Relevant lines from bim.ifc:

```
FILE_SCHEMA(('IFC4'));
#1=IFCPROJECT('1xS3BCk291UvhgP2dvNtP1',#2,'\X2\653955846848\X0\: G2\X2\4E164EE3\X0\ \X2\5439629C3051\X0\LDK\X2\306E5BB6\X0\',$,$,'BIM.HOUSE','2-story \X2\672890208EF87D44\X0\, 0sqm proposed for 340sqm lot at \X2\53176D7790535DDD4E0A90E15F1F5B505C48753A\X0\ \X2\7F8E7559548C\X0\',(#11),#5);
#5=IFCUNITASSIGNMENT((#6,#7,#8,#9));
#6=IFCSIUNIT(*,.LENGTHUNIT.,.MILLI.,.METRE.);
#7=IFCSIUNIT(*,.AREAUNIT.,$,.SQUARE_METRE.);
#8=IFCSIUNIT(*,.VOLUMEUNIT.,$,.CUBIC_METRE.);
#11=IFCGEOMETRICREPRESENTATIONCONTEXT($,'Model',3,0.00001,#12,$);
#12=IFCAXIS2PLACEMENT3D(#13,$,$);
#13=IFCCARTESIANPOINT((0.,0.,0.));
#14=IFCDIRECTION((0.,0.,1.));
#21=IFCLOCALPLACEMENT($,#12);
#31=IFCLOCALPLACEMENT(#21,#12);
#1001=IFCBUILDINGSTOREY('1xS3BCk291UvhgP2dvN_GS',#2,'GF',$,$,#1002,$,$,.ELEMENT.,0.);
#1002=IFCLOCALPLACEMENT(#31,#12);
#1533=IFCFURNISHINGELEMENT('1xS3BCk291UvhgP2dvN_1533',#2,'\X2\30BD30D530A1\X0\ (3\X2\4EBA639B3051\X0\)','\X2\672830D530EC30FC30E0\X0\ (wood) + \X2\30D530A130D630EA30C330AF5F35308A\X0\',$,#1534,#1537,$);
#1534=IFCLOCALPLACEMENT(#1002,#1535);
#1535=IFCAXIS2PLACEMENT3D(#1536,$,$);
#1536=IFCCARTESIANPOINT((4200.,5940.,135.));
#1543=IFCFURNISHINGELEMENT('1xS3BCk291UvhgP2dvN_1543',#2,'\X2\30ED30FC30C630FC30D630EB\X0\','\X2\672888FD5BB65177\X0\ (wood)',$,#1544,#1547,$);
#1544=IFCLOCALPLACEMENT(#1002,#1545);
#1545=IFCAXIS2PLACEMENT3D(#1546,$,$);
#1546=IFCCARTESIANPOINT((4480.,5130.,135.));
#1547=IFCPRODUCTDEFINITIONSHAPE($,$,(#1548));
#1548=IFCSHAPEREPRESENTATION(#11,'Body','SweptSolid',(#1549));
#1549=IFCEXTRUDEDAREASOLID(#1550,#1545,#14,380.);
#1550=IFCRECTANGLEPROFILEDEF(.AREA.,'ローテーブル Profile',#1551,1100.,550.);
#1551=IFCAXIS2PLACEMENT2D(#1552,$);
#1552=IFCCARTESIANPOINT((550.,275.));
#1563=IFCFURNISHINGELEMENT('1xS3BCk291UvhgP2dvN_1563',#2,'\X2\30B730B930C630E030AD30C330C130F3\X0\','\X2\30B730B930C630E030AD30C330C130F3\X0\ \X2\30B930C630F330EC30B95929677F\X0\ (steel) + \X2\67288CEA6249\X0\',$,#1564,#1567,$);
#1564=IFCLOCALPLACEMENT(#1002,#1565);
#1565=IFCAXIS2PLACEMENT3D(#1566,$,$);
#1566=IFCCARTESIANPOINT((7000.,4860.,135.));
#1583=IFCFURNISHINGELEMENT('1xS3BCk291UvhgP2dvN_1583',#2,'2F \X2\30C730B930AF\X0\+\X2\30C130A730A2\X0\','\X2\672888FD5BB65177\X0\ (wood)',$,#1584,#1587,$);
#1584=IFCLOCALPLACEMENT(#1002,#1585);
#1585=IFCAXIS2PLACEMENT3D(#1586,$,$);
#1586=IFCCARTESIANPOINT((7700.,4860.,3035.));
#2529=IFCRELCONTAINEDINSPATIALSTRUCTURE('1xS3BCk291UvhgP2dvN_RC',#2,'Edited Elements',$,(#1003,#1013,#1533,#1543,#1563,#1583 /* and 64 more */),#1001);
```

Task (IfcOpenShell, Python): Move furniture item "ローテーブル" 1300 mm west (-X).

```python
import ifcopenshell
import ifcopenshell.api.geometry
import ifcopenshell.util.placement
import ifcopenshell.util.unit

model = ifcopenshell.open("bim.ifc")
unit_scale = ifcopenshell.util.unit.calculate_unit_scale(model)

item = model.by_guid("1xS3BCk291UvhgP2dvN_1543")
matrix = ifcopenshell.util.placement.get_local_placement(item.ObjectPlacement)
matrix[0, 3] -= 1.3 / unit_scale
ifcopenshell.api.geometry.edit_object_placement(model, product=item, matrix=matrix, is_si=False)

print(ifcopenshell.util.placement.get_local_placement(item.ObjectPlacement).round(3) + 0.0)

model.write("bim-out.ifc")
```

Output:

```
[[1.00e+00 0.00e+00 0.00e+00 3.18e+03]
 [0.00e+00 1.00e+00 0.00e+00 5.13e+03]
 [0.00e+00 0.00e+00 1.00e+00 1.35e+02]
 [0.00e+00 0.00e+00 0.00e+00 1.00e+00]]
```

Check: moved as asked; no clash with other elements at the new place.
